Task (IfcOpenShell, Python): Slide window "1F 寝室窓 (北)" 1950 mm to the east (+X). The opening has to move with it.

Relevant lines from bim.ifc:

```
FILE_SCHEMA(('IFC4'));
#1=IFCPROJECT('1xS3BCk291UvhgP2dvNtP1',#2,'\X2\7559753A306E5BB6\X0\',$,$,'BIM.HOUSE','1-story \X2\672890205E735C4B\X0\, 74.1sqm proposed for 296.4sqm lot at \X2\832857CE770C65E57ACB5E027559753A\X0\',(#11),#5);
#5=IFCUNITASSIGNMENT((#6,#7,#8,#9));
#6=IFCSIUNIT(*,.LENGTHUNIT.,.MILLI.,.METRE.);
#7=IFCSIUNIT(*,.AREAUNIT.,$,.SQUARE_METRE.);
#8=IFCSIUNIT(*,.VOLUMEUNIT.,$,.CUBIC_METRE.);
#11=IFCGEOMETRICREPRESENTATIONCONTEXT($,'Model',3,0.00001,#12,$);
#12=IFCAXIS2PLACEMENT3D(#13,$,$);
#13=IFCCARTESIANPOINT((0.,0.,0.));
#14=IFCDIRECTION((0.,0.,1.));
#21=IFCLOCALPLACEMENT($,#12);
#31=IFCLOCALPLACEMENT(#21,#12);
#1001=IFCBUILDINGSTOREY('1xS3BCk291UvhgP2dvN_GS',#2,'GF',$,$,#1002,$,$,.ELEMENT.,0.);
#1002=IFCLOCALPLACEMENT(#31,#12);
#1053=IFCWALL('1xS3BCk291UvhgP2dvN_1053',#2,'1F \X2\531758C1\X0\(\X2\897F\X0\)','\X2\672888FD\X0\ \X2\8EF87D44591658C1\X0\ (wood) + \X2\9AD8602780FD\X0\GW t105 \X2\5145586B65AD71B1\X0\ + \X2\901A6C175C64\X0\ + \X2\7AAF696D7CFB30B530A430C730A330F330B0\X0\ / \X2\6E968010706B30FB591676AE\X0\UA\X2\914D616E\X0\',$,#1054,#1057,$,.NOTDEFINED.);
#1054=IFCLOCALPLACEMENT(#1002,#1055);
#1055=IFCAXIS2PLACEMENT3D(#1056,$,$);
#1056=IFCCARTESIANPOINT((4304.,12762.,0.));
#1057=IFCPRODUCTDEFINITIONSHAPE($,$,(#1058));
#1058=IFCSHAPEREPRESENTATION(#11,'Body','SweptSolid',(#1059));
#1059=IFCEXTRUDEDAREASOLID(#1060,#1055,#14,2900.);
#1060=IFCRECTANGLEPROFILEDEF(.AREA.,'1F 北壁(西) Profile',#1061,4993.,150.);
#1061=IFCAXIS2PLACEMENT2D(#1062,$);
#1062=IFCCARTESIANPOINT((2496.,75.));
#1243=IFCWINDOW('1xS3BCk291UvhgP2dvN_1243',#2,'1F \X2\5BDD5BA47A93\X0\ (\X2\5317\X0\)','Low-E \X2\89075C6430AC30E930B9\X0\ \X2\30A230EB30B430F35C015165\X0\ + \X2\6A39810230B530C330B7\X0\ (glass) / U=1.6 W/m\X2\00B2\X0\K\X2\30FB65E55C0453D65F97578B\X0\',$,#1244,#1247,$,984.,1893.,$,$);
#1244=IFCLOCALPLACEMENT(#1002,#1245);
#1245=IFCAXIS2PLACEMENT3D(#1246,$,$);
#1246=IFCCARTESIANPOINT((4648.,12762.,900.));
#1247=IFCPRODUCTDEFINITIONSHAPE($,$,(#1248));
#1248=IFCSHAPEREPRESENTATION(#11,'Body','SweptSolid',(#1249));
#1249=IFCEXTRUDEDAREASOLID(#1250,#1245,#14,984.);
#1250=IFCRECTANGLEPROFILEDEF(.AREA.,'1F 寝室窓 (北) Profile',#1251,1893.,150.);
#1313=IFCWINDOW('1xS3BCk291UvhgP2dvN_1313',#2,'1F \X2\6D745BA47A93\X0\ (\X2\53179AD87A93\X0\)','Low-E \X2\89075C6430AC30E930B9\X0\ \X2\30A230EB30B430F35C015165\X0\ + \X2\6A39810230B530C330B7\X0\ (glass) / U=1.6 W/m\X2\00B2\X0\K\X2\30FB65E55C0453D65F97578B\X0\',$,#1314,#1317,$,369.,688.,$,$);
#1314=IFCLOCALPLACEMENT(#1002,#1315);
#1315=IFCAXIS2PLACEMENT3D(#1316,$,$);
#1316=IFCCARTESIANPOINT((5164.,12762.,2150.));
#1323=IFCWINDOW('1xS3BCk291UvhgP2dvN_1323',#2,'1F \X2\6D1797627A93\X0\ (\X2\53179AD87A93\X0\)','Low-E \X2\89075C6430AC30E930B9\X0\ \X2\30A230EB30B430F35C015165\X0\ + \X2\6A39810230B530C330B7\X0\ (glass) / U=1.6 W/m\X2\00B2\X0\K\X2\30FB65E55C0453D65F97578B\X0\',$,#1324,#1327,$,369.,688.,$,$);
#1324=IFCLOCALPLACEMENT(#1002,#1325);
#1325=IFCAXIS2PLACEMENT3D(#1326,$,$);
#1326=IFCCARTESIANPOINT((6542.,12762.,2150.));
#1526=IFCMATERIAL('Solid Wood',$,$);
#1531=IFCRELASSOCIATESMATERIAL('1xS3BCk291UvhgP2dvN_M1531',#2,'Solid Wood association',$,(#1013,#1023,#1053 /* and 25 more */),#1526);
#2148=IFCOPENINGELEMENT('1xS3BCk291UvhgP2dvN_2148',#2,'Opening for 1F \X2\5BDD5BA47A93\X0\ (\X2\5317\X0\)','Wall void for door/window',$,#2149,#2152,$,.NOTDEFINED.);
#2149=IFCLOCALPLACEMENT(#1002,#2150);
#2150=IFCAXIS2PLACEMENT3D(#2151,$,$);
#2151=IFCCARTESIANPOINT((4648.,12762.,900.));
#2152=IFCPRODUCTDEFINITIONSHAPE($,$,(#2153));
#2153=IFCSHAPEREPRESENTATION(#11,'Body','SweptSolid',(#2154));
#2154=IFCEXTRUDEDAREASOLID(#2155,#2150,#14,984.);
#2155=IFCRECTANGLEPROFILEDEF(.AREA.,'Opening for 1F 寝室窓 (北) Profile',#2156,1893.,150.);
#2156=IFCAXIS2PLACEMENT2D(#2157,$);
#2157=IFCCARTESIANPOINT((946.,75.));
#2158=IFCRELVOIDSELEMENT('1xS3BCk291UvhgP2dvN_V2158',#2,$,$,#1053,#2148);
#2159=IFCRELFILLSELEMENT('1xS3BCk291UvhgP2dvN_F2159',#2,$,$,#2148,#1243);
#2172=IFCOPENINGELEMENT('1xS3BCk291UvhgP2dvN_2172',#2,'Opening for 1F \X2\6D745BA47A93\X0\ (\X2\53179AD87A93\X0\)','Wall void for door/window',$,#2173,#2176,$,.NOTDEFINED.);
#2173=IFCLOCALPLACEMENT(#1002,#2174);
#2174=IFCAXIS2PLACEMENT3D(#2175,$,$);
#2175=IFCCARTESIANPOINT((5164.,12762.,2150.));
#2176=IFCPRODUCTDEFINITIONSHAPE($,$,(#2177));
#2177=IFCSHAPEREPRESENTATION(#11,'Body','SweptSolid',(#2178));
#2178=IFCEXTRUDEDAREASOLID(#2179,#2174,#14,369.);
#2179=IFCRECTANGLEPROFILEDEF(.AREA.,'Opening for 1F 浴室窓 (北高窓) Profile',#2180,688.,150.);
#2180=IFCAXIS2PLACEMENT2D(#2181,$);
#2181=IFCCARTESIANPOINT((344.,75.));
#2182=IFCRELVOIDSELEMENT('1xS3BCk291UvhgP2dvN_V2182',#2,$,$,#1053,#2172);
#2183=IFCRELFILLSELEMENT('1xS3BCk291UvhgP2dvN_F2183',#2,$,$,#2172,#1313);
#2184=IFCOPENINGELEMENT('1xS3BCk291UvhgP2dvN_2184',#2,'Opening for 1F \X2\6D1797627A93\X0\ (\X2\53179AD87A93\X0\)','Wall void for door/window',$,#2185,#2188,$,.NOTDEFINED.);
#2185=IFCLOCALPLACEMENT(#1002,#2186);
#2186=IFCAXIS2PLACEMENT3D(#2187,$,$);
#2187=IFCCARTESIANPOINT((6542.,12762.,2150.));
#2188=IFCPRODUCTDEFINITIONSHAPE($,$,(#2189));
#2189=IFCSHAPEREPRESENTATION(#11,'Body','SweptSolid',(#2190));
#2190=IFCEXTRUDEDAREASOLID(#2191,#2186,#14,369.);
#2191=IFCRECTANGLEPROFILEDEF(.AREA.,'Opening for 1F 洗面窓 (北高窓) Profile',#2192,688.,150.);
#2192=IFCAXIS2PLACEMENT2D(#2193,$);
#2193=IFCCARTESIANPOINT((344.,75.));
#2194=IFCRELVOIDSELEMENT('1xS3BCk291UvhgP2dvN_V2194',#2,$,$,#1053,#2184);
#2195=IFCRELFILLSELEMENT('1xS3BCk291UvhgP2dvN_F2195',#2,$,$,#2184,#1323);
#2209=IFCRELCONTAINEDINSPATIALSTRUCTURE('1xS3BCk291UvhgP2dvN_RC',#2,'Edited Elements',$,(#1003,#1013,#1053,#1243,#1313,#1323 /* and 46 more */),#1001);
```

```python
import ifcopenshell
import ifcopenshell.api.geometry
import ifcopenshell.util.placement

model = ifcopenshell.open("bim.ifc")

window = model.by_guid("1xS3BCk291UvhgP2dvN_1243")
opening = window.FillsVoids[0].RelatingOpeningElement
wall = opening.VoidsElements[0].RelatingBuildingElement

wall_matrix = ifcopenshell.util.placement.get_local_placement(wall.ObjectPlacement)
shift = wall_matrix[:3, 0] * 1950.0
before = ifcopenshell.util.placement.get_local_placement(window.ObjectPlacement)[:3, 3].copy()

# The window is not placed relative to its opening, so move both.
for product in (opening, window):
    matrix = ifcopenshell.util.placement.get_local_placement(product.ObjectPlacement)
    matrix[:3, 3] += shift
    ifcopenshell.api.geometry.edit_object_placement(model, product=product, matrix=matrix, is_si=False)

after = ifcopenshell.util.placement.get_local_placement(window.ObjectPlacement)[:3, 3]
print("window moved by", (after - before).round(3) + 0.0)

model.write("bim_v2.ifc")
```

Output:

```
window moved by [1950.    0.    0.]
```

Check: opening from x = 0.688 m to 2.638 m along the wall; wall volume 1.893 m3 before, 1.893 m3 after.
